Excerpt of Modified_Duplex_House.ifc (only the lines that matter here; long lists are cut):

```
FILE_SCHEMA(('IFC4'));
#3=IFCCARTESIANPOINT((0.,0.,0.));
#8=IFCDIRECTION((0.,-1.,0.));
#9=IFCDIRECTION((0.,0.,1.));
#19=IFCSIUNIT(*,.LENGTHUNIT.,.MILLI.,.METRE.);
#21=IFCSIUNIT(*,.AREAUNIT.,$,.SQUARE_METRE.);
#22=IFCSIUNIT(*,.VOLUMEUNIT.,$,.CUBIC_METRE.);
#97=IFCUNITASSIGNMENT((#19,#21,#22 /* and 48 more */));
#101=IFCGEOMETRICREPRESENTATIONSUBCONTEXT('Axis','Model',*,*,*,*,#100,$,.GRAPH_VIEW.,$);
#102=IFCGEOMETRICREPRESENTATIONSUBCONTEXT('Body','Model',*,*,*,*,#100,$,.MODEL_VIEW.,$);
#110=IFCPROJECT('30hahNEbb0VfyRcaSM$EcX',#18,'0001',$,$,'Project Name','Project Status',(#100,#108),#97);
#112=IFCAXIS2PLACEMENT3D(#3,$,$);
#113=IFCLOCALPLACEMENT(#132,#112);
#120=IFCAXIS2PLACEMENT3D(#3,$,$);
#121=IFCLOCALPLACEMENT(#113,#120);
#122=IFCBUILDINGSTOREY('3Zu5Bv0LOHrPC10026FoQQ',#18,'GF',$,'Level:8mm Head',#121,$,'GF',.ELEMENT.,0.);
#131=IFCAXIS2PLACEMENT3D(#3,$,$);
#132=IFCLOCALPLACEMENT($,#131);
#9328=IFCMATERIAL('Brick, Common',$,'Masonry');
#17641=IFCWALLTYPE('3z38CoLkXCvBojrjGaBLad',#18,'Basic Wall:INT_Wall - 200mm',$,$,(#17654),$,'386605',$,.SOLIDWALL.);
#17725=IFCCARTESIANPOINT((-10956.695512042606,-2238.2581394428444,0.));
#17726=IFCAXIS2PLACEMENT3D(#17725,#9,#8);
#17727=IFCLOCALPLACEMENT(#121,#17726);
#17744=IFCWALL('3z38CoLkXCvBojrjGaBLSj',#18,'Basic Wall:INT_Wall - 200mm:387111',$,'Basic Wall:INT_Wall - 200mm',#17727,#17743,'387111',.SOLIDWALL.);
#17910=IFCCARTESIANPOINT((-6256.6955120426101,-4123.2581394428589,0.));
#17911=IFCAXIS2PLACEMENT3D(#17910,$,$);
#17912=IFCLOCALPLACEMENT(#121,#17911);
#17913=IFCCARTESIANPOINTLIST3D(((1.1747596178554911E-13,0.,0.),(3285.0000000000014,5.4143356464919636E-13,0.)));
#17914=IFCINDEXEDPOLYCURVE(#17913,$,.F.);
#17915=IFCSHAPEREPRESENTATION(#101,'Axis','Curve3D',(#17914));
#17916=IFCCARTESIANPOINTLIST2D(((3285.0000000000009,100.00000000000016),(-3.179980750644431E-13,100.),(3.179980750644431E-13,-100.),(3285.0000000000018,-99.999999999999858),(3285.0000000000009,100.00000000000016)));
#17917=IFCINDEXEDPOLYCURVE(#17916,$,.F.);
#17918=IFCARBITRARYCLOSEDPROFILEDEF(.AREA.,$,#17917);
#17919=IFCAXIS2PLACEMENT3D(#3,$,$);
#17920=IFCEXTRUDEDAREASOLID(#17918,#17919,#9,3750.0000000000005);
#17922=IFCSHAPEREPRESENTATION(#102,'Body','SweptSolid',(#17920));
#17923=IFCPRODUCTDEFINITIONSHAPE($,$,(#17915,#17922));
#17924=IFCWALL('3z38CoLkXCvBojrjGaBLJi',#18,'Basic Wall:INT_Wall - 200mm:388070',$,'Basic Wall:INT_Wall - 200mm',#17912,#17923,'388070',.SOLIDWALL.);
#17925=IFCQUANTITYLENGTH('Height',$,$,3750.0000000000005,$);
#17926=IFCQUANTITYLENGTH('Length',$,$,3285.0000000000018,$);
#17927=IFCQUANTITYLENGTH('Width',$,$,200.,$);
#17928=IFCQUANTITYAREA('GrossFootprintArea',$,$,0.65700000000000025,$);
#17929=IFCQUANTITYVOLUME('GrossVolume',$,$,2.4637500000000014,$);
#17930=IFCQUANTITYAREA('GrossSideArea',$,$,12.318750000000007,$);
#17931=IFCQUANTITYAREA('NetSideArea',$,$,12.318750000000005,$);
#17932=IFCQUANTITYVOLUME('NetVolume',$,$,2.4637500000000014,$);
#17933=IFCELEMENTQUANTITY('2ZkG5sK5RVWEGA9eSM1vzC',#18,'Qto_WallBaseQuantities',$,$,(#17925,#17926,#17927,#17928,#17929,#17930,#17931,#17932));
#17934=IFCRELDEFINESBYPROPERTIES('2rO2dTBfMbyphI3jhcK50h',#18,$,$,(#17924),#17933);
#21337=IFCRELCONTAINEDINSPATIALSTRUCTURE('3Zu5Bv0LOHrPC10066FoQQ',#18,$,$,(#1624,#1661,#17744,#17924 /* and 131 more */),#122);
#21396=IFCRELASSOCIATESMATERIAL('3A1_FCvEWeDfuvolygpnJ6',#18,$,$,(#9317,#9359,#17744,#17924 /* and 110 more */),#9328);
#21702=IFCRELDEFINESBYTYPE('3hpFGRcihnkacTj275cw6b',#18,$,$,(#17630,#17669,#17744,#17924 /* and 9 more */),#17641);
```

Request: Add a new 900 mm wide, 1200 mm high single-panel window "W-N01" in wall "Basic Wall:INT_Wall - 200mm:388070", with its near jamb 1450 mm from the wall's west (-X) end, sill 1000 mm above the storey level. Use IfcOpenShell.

```python
import numpy as np
import ifcopenshell
import ifcopenshell.api.feature
import ifcopenshell.api.geometry
import ifcopenshell.api.pset
import ifcopenshell.api.root
import ifcopenshell.api.spatial
import ifcopenshell.geom
import ifcopenshell.util.element
import ifcopenshell.util.placement
import ifcopenshell.util.representation
import ifcopenshell.util.shape
import ifcopenshell.util.unit

model = ifcopenshell.open("Modified_Duplex_House.ifc")
unit_scale = ifcopenshell.util.unit.calculate_unit_scale(model)
area_scale = ifcopenshell.util.unit.calculate_unit_scale(model, "AREAUNIT")
volume_scale = ifcopenshell.util.unit.calculate_unit_scale(model, "VOLUMEUNIT")
settings = ifcopenshell.geom.settings()


def volume(element):
    """Net volume in cubic metres, openings subtracted."""
    shape = ifcopenshell.geom.create_shape(settings, element)
    return ifcopenshell.util.shape.get_volume(shape.geometry)


wall = model.by_guid("3z38CoLkXCvBojrjGaBLJi")
storey = ifcopenshell.util.element.get_container(wall, ifc_class="IfcBuildingStorey")
context = ifcopenshell.util.representation.get_context(model, "Model", "Body", "MODEL_VIEW")
before = volume(wall)

width, height, from_end, sill = 0.9, 1.2, 1.45, 1  # metres

# The wall runs along its own X axis, and the end named is its -X end.
wall_shape = ifcopenshell.geom.create_shape(settings, wall)
x, y, z = ifcopenshell.util.shape.get_vertices(wall_shape.geometry).T
start = x.min() + from_end
face, thickness = float(y.min()), float(y.max() - y.min())
wall_matrix = ifcopenshell.util.placement.get_local_placement(wall.ObjectPlacement)
level = ifcopenshell.util.placement.get_local_placement(storey.ObjectPlacement)[2, 3]


def in_wall(x, y):
    """Placement at x, y metres in the wall's axes, at sill height."""
    matrix = wall_matrix.copy()
    matrix[:, 3] = wall_matrix @ np.array([x / unit_scale, y / unit_scale, 0.0, 1.0])
    matrix[2, 3] = level + sill / unit_scale
    return matrix


# Opening: a box that overshoots both wall faces by 50 mm.
opening = ifcopenshell.api.root.create_entity(model, ifc_class="IfcOpeningElement", predefined_type="OPENING")
box = ifcopenshell.api.geometry.add_wall_representation(
    model, context=context, length=width, height=height, thickness=thickness + 0.1
)
ifcopenshell.api.geometry.assign_representation(model, product=opening, representation=box)
ifcopenshell.api.geometry.edit_object_placement(model, product=opening, matrix=in_wall(start, face - 0.05), is_si=False)
ifcopenshell.api.feature.add_feature(model, feature=opening, element=wall)

window = ifcopenshell.api.root.create_entity(model, ifc_class="IfcWindow", name="W-N01", predefined_type="WINDOW")
window.OverallWidth, window.OverallHeight = width / unit_scale, height / unit_scale
window.PartitioningType = "SINGLE_PANEL"
body = ifcopenshell.api.geometry.add_window_representation(
    model,
    context=context,
    overall_width=window.OverallWidth,
    overall_height=window.OverallHeight,
    partition_type="SINGLE_PANEL",
)
ifcopenshell.api.geometry.assign_representation(model, product=window, representation=body)
ifcopenshell.api.spatial.assign_container(model, products=[window], relating_structure=storey)
ifcopenshell.api.feature.add_filling(model, opening=opening, element=window)

# Centre the window in the wall's thickness.
ifcopenshell.api.geometry.edit_object_placement(model, product=window, matrix=in_wall(start, face), is_si=False)
window_shape = ifcopenshell.geom.create_shape(settings, window)
depth = ifcopenshell.util.shape.get_vertices(window_shape.geometry)[:, 1]
offset = face + thickness / 2 - (depth.min() + depth.max()) / 2
ifcopenshell.api.geometry.edit_object_placement(model, product=window, matrix=in_wall(start, offset), is_si=False)

after = volume(wall)

# Update the wall's stored quantities.
qto = model.by_id(ifcopenshell.util.element.get_pset(wall, "Qto_WallBaseQuantities", should_inherit=False)["id"])
ifcopenshell.api.pset.edit_qto(model, qto=qto, properties={
    "NetSideArea": after / thickness / area_scale,
    "NetVolume": after / volume_scale,
})

print(f"wall volume {before:.3f} -> {after:.3f} m3")

model.write("Modified_Duplex_House_v2.ifc")
```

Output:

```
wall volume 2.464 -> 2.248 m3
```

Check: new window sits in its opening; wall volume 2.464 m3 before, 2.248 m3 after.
